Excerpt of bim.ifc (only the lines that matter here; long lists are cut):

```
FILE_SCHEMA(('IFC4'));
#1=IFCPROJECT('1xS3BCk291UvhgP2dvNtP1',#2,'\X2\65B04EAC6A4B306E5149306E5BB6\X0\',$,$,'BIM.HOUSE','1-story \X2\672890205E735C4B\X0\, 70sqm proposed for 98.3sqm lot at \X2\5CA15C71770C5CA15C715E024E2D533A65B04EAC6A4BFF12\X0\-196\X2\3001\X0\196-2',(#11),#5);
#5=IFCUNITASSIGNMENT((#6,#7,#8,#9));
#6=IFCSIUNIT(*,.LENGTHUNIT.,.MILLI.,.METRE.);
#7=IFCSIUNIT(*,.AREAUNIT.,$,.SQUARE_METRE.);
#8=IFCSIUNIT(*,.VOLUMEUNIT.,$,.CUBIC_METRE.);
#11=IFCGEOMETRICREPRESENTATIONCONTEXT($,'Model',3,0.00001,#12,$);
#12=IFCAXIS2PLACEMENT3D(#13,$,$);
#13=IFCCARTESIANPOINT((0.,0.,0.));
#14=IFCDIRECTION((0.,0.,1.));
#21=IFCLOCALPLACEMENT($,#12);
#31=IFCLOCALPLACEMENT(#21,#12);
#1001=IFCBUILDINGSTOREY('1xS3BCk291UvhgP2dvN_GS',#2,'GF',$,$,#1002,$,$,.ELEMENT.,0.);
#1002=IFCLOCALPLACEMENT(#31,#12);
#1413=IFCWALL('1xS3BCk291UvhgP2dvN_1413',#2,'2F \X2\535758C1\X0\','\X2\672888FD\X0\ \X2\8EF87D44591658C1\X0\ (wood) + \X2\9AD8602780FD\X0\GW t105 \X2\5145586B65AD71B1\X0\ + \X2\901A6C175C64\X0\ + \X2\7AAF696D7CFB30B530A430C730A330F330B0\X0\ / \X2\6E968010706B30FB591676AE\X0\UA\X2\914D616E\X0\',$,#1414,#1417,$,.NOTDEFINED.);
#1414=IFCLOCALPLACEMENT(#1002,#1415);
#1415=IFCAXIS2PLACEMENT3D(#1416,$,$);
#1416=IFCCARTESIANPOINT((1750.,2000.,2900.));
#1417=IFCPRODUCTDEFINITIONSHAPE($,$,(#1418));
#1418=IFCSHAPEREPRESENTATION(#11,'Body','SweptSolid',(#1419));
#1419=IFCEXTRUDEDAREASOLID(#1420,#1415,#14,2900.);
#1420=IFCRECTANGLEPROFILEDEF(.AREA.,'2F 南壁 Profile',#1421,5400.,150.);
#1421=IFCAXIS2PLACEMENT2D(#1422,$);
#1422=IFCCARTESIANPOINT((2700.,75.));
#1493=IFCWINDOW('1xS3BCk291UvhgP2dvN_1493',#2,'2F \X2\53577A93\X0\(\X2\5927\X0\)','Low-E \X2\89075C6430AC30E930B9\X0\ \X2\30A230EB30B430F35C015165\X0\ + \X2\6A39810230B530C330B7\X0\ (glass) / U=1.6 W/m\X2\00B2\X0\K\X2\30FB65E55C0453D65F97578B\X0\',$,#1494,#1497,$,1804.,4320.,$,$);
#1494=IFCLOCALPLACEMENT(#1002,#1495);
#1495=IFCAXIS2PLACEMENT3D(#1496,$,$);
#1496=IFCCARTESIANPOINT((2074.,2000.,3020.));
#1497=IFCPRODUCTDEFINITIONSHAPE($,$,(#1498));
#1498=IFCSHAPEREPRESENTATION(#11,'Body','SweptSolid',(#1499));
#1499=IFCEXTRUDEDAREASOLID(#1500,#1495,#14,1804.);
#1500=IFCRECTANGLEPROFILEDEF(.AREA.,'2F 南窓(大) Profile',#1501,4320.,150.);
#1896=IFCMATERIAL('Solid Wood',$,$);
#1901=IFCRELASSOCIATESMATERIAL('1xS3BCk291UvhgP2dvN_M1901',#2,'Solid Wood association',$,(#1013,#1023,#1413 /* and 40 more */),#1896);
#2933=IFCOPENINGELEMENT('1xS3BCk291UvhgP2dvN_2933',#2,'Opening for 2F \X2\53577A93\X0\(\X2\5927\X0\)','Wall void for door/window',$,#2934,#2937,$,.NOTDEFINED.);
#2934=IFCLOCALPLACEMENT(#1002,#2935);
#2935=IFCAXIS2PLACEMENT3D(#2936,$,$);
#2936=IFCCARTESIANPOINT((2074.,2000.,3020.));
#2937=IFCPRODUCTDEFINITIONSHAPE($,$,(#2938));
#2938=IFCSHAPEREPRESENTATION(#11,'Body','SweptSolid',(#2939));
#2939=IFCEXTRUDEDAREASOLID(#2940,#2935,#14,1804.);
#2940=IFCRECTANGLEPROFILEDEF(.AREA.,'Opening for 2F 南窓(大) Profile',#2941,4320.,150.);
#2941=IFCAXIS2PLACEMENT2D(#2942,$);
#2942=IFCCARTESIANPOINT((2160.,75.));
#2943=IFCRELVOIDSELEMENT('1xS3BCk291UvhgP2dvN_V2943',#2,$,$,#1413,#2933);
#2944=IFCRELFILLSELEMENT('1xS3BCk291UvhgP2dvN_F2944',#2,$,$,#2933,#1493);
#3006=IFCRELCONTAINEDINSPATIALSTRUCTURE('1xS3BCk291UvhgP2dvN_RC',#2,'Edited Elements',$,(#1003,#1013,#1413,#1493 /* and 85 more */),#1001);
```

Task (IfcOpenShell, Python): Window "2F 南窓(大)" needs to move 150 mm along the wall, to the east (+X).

```python
import ifcopenshell
import ifcopenshell.api.geometry
import ifcopenshell.util.placement

model = ifcopenshell.open("bim.ifc")

window = model.by_id(1493)
opening = window.FillsVoids[0].RelatingOpeningElement
wall = opening.VoidsElements[0].RelatingBuildingElement

wall_matrix = ifcopenshell.util.placement.get_local_placement(wall.ObjectPlacement)
shift = wall_matrix[:3, 0] * 150.0
before = ifcopenshell.util.placement.get_local_placement(window.ObjectPlacement)[:3, 3].copy()

# The window is not placed relative to its opening, so move both.
for product in (opening, window):
    matrix = ifcopenshell.util.placement.get_local_placement(product.ObjectPlacement)
    matrix[:3, 3] += shift
    ifcopenshell.api.geometry.edit_object_placement(model, product=product, matrix=matrix, is_si=False)

after = ifcopenshell.util.placement.get_local_placement(window.ObjectPlacement)[:3, 3]
print("window moved by", (after - before).round(3) + 0.0)

model.write("bim_v2.ifc")
```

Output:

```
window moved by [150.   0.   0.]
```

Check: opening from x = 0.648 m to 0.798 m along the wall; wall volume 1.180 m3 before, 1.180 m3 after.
